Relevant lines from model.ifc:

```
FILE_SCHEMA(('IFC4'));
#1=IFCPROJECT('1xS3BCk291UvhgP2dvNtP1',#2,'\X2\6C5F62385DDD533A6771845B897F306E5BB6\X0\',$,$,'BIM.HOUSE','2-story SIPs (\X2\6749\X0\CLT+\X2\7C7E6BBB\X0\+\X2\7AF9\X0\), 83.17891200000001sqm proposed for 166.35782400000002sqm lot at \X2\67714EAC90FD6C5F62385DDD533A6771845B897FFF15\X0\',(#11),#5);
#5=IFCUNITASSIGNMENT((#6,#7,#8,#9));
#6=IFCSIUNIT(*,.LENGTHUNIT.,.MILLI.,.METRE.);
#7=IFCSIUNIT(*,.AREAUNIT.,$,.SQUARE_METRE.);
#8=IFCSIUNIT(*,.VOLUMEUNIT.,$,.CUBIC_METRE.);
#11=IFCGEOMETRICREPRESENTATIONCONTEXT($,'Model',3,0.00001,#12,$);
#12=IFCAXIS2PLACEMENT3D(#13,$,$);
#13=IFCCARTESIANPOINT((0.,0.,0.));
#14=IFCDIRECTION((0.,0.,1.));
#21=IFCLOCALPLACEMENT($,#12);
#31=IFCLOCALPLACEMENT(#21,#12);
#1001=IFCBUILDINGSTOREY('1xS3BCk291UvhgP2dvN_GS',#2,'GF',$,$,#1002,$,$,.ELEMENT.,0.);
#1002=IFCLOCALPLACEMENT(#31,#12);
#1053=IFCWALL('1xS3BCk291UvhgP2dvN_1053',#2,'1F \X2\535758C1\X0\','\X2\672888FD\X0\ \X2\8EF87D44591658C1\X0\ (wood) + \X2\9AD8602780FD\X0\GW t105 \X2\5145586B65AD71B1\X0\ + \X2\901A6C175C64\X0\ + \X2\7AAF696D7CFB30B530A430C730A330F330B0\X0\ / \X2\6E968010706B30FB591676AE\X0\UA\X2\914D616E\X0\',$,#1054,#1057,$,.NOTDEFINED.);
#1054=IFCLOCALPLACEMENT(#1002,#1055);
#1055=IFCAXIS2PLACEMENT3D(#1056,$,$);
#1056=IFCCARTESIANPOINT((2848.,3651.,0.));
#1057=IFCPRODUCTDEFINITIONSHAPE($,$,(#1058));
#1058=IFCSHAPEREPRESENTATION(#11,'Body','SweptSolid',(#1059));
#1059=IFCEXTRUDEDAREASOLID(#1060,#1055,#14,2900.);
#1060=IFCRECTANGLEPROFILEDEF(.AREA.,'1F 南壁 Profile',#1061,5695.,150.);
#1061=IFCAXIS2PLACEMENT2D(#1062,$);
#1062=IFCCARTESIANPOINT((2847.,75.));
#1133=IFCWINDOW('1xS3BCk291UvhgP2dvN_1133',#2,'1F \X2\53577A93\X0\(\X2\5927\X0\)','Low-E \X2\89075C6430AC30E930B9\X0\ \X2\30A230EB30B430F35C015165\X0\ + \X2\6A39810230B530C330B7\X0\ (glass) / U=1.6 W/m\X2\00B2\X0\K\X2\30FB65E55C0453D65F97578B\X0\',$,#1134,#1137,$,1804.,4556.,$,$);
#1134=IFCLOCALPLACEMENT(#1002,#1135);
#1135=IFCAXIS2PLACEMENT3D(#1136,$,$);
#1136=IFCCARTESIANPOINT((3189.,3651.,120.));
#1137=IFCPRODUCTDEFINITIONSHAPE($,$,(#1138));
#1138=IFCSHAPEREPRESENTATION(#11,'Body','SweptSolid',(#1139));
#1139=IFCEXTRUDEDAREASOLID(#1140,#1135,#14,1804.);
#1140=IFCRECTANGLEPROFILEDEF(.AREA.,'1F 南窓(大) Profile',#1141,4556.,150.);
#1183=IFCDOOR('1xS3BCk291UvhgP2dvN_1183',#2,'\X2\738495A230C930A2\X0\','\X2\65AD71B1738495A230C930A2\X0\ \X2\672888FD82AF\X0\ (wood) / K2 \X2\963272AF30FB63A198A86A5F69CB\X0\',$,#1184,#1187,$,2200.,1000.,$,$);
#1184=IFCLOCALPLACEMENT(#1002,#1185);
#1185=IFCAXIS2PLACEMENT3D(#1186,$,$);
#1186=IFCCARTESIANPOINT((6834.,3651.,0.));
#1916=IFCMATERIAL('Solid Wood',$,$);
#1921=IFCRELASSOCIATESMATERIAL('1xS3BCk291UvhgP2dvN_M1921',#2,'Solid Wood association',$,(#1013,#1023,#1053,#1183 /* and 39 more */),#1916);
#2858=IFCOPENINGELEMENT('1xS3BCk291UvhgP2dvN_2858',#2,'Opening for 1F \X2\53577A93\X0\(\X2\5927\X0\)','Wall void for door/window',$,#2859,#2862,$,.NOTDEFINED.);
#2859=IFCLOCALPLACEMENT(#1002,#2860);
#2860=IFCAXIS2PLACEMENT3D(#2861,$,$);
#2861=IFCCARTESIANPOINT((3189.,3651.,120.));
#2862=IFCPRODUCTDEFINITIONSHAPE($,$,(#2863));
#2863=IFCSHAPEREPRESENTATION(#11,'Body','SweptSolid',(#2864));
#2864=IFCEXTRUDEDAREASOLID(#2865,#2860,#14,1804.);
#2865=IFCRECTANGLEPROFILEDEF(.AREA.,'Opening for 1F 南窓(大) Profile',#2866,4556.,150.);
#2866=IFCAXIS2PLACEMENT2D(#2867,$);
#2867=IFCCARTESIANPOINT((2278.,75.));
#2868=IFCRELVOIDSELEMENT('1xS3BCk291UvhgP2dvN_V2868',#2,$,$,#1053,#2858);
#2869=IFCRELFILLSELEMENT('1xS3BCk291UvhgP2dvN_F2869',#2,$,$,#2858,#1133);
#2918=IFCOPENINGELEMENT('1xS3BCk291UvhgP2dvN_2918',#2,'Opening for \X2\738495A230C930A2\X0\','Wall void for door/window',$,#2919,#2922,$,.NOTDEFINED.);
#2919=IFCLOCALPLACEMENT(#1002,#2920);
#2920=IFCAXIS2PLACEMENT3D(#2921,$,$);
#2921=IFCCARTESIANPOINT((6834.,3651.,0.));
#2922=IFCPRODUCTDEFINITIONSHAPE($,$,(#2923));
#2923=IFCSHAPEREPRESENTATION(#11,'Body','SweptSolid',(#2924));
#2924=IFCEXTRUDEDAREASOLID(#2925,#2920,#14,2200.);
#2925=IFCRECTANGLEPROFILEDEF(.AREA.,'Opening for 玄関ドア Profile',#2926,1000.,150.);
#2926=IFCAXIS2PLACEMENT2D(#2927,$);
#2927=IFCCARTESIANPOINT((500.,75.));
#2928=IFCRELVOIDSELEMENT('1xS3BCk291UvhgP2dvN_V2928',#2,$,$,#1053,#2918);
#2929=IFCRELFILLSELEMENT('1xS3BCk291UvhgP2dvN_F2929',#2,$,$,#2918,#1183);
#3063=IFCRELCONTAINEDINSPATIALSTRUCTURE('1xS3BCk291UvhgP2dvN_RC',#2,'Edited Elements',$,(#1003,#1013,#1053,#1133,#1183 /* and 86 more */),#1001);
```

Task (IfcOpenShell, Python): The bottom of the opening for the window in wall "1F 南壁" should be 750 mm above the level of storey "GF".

```python
import numpy as np
import ifcopenshell
import ifcopenshell.api.geometry
import ifcopenshell.geom
import ifcopenshell.util.element
import ifcopenshell.util.placement
import ifcopenshell.util.shape
import ifcopenshell.util.unit

model = ifcopenshell.open("model.ifc")
unit_scale = ifcopenshell.util.unit.calculate_unit_scale(model)

window = model.by_id(1133)
opening = window.FillsVoids[0].RelatingOpeningElement
storey = ifcopenshell.util.element.get_container(window, ifc_class="IfcBuildingStorey")
level = ifcopenshell.util.placement.get_local_placement(storey.ObjectPlacement)[2, 3]

# The opening's origin need not be at the sill, so measure its lowest point.
shape = ifcopenshell.geom.create_shape(ifcopenshell.geom.settings(), opening)
bottom = ifcopenshell.util.shape.get_shape_bottom_elevation(shape, shape.geometry) / unit_scale
dz = level + 0.75 / unit_scale - bottom

shift = np.array([0.0, 0.0, dz])
# The window is not placed relative to its opening, so move both.
for product in (opening, window):
    matrix = ifcopenshell.util.placement.get_local_placement(product.ObjectPlacement)
    matrix[:3, 3] += shift
    ifcopenshell.api.geometry.edit_object_placement(model, product=product, matrix=matrix, is_si=False)

print(f"moved by {dz * unit_scale:+.3f} m")

model.write("model_updated.ifc")
```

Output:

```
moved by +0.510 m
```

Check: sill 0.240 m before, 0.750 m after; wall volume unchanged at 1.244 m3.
